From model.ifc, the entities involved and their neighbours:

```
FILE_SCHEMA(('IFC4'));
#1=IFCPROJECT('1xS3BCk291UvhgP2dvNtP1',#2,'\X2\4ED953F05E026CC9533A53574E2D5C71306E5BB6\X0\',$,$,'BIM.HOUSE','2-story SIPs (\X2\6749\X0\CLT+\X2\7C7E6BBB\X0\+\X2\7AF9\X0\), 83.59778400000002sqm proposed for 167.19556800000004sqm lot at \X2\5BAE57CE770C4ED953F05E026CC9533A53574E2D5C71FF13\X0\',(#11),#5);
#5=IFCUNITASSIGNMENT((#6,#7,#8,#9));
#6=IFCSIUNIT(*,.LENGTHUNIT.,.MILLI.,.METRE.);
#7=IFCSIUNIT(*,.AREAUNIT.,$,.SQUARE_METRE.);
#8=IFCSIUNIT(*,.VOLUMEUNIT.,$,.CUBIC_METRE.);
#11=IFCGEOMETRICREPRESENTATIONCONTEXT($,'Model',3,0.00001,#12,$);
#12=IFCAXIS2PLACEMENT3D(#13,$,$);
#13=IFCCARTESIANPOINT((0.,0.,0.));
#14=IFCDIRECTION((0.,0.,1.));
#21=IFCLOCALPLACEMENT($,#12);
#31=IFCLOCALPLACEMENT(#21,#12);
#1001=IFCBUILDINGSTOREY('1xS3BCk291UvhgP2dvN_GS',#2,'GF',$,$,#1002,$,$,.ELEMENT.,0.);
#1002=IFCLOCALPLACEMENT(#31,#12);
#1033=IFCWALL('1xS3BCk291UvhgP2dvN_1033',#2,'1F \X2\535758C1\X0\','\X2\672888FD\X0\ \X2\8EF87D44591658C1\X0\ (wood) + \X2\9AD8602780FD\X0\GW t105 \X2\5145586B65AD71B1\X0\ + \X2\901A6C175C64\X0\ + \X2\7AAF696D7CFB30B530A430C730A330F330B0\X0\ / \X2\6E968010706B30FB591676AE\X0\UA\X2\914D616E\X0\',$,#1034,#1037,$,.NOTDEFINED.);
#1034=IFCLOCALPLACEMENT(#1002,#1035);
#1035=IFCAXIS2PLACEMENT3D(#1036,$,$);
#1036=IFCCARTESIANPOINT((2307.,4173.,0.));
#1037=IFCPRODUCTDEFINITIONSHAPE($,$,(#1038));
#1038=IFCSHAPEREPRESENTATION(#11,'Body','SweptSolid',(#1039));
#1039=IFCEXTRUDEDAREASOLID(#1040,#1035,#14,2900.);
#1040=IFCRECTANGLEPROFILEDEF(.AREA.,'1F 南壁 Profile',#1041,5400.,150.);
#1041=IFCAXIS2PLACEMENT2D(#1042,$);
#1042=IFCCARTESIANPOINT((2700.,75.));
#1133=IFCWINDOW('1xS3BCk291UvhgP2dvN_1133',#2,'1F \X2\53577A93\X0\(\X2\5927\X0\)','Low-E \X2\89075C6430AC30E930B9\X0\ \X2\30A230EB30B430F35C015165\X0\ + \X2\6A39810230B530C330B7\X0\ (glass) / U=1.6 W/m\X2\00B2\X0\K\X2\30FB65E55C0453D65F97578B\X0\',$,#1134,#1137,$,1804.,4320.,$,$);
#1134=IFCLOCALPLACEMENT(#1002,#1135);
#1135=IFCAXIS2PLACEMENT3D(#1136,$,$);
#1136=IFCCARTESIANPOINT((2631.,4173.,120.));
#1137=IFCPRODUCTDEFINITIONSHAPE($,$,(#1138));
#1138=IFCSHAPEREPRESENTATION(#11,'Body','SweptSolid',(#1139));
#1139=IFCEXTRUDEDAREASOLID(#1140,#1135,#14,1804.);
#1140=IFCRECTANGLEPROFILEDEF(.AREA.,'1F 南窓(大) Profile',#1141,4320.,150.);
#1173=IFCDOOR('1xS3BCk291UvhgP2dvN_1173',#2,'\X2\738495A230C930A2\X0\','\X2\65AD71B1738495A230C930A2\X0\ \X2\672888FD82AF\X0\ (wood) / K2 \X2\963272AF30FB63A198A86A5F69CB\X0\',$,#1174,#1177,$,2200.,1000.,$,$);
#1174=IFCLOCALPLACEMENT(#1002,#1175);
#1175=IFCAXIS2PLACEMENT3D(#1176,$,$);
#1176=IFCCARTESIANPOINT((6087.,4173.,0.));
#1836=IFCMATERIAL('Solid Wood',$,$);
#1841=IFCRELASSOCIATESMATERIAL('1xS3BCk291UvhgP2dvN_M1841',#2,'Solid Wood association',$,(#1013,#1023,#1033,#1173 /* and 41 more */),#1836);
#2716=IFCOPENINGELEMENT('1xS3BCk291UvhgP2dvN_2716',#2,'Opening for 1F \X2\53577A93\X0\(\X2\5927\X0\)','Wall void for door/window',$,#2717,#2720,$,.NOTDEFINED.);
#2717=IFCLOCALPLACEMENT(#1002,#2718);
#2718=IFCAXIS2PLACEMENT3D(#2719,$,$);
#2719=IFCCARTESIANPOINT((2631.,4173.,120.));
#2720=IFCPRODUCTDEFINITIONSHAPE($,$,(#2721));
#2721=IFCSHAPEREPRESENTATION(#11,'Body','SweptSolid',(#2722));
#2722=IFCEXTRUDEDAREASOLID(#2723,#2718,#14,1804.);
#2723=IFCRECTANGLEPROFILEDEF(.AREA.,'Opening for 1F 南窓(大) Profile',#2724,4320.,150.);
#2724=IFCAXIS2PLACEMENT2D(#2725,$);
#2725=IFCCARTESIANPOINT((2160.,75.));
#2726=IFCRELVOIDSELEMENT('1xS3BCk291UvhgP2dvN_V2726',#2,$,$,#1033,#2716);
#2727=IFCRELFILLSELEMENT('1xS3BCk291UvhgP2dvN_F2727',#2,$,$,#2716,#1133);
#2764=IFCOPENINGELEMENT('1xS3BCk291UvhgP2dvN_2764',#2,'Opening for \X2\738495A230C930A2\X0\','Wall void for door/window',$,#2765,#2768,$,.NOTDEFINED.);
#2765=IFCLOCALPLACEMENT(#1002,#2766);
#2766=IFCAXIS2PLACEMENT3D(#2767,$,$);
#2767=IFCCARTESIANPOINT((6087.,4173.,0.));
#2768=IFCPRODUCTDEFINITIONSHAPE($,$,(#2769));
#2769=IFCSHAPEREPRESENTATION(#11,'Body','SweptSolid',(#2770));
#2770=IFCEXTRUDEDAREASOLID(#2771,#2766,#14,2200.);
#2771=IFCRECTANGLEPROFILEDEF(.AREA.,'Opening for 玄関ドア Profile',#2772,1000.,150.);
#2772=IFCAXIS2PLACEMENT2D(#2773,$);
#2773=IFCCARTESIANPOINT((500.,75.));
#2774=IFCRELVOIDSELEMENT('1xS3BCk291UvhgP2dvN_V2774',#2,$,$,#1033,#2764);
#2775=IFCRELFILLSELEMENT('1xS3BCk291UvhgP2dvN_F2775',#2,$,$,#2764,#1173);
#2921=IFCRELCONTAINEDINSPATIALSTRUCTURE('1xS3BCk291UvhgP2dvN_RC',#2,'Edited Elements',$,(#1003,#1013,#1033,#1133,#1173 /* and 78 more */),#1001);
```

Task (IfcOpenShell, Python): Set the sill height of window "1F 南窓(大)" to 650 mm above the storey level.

```python
import numpy as np
import ifcopenshell
import ifcopenshell.api.geometry
import ifcopenshell.geom
import ifcopenshell.util.element
import ifcopenshell.util.placement
import ifcopenshell.util.shape
import ifcopenshell.util.unit

model = ifcopenshell.open("model.ifc")
unit_scale = ifcopenshell.util.unit.calculate_unit_scale(model)

window = model.by_guid("1xS3BCk291UvhgP2dvN_1133")
opening = window.FillsVoids[0].RelatingOpeningElement
storey = ifcopenshell.util.element.get_container(window, ifc_class="IfcBuildingStorey")
level = ifcopenshell.util.placement.get_local_placement(storey.ObjectPlacement)[2, 3]

# The opening's origin need not be at the sill, so measure its lowest point.
shape = ifcopenshell.geom.create_shape(ifcopenshell.geom.settings(), opening)
bottom = ifcopenshell.util.shape.get_shape_bottom_elevation(shape, shape.geometry) / unit_scale
dz = level + 0.65 / unit_scale - bottom

shift = np.array([0.0, 0.0, dz])
# The window is not placed relative to its opening, so move both.
for product in (opening, window):
    matrix = ifcopenshell.util.placement.get_local_placement(product.ObjectPlacement)
    matrix[:3, 3] += shift
    ifcopenshell.api.geometry.edit_object_placement(model, product=product, matrix=matrix, is_si=False)

print(f"moved by {dz * unit_scale:+.3f} m")

model.write("model_updated.ifc")
```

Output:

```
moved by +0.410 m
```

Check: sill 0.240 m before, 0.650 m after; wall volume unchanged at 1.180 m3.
